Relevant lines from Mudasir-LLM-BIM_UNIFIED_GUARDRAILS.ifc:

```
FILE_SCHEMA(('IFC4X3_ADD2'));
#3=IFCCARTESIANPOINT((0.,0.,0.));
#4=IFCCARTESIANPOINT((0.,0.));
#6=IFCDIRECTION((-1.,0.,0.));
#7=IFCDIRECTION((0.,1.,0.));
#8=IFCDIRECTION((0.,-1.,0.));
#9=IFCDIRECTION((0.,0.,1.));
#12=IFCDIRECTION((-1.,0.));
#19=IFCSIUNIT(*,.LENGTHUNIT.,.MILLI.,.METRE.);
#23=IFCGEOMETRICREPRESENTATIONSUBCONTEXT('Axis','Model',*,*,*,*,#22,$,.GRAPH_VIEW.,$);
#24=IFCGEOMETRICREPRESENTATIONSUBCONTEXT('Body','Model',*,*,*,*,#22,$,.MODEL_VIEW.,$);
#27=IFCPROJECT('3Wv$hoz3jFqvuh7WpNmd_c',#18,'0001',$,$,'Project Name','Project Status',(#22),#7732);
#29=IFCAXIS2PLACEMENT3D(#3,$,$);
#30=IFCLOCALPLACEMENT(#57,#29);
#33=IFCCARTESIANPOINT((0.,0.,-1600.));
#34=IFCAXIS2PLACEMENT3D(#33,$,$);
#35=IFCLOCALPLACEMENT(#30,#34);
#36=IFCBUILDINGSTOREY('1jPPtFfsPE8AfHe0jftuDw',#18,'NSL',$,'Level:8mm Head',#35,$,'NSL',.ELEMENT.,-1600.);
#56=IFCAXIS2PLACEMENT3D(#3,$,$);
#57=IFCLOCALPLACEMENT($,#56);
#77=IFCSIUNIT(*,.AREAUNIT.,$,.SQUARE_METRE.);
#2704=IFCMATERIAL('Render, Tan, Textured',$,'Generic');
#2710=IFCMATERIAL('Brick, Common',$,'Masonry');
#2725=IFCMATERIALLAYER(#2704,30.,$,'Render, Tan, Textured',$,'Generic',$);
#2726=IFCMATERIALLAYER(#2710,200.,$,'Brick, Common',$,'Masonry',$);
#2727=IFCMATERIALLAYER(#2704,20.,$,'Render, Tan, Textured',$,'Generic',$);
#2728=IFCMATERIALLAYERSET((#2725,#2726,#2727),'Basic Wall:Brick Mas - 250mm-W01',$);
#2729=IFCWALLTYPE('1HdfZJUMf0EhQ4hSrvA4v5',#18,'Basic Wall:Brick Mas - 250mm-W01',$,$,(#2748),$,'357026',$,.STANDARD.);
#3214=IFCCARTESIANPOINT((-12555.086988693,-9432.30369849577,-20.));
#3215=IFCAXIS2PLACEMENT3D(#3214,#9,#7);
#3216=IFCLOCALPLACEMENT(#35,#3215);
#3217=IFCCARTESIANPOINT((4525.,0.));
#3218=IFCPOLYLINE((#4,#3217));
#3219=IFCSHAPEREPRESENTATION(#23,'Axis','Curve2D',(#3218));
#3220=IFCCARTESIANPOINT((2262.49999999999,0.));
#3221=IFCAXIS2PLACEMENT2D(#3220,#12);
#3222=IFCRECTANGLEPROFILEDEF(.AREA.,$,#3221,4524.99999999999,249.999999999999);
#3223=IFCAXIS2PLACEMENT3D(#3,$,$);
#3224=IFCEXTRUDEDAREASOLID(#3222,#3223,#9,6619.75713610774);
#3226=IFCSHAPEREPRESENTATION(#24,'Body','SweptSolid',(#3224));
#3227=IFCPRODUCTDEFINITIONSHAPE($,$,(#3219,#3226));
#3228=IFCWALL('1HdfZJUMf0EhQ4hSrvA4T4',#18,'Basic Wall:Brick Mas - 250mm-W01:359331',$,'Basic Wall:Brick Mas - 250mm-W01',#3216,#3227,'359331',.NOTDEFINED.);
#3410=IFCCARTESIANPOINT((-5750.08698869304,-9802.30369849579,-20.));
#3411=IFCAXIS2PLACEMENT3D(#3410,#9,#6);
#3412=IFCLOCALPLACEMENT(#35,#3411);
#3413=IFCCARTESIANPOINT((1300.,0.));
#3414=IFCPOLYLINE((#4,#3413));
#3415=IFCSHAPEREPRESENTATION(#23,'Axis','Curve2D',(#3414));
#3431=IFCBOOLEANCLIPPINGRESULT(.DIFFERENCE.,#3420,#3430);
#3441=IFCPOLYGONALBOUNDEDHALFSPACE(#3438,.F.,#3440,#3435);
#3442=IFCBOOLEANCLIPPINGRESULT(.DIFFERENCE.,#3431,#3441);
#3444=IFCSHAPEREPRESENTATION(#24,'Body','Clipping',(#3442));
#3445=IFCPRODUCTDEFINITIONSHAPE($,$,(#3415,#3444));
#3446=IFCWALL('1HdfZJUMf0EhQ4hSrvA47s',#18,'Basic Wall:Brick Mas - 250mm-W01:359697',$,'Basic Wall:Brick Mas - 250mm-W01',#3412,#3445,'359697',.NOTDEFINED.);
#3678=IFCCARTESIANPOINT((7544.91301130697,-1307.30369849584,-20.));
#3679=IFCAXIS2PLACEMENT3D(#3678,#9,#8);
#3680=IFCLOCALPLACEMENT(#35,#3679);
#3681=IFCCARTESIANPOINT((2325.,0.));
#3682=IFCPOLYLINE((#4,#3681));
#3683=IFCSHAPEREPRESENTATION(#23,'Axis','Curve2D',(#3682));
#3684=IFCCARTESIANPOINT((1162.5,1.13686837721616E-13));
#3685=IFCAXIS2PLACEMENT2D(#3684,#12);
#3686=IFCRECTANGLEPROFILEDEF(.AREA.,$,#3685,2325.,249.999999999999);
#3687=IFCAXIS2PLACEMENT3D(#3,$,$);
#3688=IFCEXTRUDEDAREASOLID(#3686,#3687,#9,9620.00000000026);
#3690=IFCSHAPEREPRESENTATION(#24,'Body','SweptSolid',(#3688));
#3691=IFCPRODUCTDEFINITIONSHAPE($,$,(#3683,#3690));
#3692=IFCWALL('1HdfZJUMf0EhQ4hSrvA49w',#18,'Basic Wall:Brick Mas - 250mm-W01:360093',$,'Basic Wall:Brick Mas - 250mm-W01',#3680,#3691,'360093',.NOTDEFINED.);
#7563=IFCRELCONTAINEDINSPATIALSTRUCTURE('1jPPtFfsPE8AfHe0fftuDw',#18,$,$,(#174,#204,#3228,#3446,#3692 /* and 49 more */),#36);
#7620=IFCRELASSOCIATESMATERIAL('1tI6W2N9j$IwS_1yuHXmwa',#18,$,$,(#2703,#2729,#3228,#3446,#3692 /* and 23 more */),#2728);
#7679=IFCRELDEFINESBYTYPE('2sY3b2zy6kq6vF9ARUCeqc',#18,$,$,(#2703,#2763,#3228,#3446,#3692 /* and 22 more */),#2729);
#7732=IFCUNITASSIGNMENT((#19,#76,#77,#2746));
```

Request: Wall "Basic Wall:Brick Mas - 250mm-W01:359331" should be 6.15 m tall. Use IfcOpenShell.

```python
import ifcopenshell
import ifcopenshell.geom
import ifcopenshell.util.representation
import ifcopenshell.util.shape
import ifcopenshell.util.unit

model = ifcopenshell.open("Mudasir-LLM-BIM_UNIFIED_GUARDRAILS.ifc")
unit_scale = ifcopenshell.util.unit.calculate_unit_scale(model)
settings = ifcopenshell.geom.settings()


def volume(element):
    """Net volume in cubic metres, openings subtracted."""
    shape = ifcopenshell.geom.create_shape(settings, element)
    return ifcopenshell.util.shape.get_volume(shape.geometry)


wall = model.by_id(3228)
before = volume(wall)

body = ifcopenshell.util.representation.get_representation(wall, "Model", "Body")
solid = body.Items[0]
old_height = solid.Depth
solid.Depth = 6.15 / unit_scale
after = volume(wall)

print(f"height {old_height:g} -> {solid.Depth:g}, volume {before:.3f} -> {after:.3f} m3")

model.write("Mudasir-LLM-BIM_UNIFIED_GUARDRAILS-out.ifc")
```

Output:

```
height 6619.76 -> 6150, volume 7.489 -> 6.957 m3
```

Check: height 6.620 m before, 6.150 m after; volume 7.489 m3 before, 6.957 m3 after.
